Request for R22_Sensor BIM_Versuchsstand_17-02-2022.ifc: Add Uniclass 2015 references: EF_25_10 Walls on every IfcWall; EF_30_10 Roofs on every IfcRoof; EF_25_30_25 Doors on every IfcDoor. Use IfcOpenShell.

First a look at what the model holds.

```python
import ifcopenshell

model = ifcopenshell.open("R22_Sensor BIM_Versuchsstand_17-02-2022.ifc")
print(model.schema)
print("classifications:", [c.Name for c in model.by_type("IfcClassification")])
for ifc_class in ("IfcDoor", "IfcRoof", "IfcStair", "IfcWall", "IfcWindow"):
    print(ifc_class, len(model.by_type(ifc_class)))
```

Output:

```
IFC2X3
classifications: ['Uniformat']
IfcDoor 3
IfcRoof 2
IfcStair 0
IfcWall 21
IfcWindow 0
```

```python
import ifcopenshell
import ifcopenshell.api.classification

model = ifcopenshell.open("R22_Sensor BIM_Versuchsstand_17-02-2022.ifc")

# IFC2X3 requires Source and Edition and has no link from the project to the system.
system = model.create_entity("IfcClassification", Source="NBS", Edition="2015", Name="Uniclass 2015")

codes = {
    "IfcWall": ("EF_25_10", "Walls"),
    "IfcRoof": ("EF_30_10", "Roofs"),
    "IfcDoor": ("EF_25_30_25", "Doors"),
}
for ifc_class, (code, name) in codes.items():
    products = model.by_type(ifc_class)
    ifcopenshell.api.classification.add_reference(
        model, products=products, classification=system, identification=code, name=name
    )
    print(code, len(products))

model.write("R22_Sensor BIM_Versuchsstand_17-02-2022_updated.ifc")
```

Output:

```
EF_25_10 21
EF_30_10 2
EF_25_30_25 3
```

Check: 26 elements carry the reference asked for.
